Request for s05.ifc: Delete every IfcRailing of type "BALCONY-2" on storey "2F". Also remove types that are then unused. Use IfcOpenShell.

First a look at what the model holds.

```python
import ifcopenshell
import ifcopenshell.util.element

model = ifcopenshell.open("s05.ifc")
print(model.schema)
storey = next(s for s in model.by_type("IfcBuildingStorey") if s.Name == "2F")
railings = [e for e in ifcopenshell.util.element.get_decomposition(storey) if e.is_a("IfcRailing")]
seen = {}
for e in railings:
    element_type = ifcopenshell.util.element.get_type(e)
    name = element_type.Name if element_type not in (None, e) else None
    seen[name] = seen.get(name, 0) + 1
for name, count in sorted(seen.items(), key=str):
    print(count, "x", name)
```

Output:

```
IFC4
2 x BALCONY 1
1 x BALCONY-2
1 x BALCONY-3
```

```python
import ifcopenshell
import ifcopenshell.api.root
import ifcopenshell.util.element

model = ifcopenshell.open("s05.ifc")

storey = next(s for s in model.by_type("IfcBuildingStorey") if s.Name == "2F")
railings = [e for e in ifcopenshell.util.element.get_decomposition(storey) if e.is_a("IfcRailing")]
targets = [e for e in railings if (t := ifcopenshell.util.element.get_type(e)) not in (None, e) and t.Name == "BALCONY-2"]
types = {ifcopenshell.util.element.get_type(e) for e in targets} - {None, *targets}

for e in targets:
    ifcopenshell.api.root.remove_product(model, product=e)
print(len(targets), "removed")

unused = [t for t in types if not ifcopenshell.util.element.get_types(t)]
for t in unused:
    ifcopenshell.api.root.remove_product(model, product=t)
print(len(unused), "unused types removed")

model.write("s05-out.ifc")
```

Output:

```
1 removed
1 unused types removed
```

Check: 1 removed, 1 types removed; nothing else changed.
